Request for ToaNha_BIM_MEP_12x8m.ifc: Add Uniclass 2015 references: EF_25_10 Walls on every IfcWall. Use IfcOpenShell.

First a look at what the model holds.

```python
import ifcopenshell

model = ifcopenshell.open("ToaNha_BIM_MEP_12x8m.ifc")
print(model.schema)
print("classifications:", [c.Name for c in model.by_type("IfcClassification")])
for ifc_class in ("IfcDoor", "IfcRoof", "IfcStair", "IfcWall", "IfcWindow"):
    print(ifc_class, len(model.by_type(ifc_class)))
```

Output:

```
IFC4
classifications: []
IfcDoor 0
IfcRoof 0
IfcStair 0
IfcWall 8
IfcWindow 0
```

```python
import ifcopenshell
import ifcopenshell.api.classification

model = ifcopenshell.open("ToaNha_BIM_MEP_12x8m.ifc")

system = ifcopenshell.api.classification.add_classification(model, classification="Uniclass 2015")

codes = {
    "IfcWall": ("EF_25_10", "Walls"),
}
for ifc_class, (code, name) in codes.items():
    products = model.by_type(ifc_class)
    ifcopenshell.api.classification.add_reference(
        model, products=products, classification=system, identification=code, name=name
    )
    print(code, len(products))

model.write("ToaNha_BIM_MEP_12x8m_updated.ifc")
```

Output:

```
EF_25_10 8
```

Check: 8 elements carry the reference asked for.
